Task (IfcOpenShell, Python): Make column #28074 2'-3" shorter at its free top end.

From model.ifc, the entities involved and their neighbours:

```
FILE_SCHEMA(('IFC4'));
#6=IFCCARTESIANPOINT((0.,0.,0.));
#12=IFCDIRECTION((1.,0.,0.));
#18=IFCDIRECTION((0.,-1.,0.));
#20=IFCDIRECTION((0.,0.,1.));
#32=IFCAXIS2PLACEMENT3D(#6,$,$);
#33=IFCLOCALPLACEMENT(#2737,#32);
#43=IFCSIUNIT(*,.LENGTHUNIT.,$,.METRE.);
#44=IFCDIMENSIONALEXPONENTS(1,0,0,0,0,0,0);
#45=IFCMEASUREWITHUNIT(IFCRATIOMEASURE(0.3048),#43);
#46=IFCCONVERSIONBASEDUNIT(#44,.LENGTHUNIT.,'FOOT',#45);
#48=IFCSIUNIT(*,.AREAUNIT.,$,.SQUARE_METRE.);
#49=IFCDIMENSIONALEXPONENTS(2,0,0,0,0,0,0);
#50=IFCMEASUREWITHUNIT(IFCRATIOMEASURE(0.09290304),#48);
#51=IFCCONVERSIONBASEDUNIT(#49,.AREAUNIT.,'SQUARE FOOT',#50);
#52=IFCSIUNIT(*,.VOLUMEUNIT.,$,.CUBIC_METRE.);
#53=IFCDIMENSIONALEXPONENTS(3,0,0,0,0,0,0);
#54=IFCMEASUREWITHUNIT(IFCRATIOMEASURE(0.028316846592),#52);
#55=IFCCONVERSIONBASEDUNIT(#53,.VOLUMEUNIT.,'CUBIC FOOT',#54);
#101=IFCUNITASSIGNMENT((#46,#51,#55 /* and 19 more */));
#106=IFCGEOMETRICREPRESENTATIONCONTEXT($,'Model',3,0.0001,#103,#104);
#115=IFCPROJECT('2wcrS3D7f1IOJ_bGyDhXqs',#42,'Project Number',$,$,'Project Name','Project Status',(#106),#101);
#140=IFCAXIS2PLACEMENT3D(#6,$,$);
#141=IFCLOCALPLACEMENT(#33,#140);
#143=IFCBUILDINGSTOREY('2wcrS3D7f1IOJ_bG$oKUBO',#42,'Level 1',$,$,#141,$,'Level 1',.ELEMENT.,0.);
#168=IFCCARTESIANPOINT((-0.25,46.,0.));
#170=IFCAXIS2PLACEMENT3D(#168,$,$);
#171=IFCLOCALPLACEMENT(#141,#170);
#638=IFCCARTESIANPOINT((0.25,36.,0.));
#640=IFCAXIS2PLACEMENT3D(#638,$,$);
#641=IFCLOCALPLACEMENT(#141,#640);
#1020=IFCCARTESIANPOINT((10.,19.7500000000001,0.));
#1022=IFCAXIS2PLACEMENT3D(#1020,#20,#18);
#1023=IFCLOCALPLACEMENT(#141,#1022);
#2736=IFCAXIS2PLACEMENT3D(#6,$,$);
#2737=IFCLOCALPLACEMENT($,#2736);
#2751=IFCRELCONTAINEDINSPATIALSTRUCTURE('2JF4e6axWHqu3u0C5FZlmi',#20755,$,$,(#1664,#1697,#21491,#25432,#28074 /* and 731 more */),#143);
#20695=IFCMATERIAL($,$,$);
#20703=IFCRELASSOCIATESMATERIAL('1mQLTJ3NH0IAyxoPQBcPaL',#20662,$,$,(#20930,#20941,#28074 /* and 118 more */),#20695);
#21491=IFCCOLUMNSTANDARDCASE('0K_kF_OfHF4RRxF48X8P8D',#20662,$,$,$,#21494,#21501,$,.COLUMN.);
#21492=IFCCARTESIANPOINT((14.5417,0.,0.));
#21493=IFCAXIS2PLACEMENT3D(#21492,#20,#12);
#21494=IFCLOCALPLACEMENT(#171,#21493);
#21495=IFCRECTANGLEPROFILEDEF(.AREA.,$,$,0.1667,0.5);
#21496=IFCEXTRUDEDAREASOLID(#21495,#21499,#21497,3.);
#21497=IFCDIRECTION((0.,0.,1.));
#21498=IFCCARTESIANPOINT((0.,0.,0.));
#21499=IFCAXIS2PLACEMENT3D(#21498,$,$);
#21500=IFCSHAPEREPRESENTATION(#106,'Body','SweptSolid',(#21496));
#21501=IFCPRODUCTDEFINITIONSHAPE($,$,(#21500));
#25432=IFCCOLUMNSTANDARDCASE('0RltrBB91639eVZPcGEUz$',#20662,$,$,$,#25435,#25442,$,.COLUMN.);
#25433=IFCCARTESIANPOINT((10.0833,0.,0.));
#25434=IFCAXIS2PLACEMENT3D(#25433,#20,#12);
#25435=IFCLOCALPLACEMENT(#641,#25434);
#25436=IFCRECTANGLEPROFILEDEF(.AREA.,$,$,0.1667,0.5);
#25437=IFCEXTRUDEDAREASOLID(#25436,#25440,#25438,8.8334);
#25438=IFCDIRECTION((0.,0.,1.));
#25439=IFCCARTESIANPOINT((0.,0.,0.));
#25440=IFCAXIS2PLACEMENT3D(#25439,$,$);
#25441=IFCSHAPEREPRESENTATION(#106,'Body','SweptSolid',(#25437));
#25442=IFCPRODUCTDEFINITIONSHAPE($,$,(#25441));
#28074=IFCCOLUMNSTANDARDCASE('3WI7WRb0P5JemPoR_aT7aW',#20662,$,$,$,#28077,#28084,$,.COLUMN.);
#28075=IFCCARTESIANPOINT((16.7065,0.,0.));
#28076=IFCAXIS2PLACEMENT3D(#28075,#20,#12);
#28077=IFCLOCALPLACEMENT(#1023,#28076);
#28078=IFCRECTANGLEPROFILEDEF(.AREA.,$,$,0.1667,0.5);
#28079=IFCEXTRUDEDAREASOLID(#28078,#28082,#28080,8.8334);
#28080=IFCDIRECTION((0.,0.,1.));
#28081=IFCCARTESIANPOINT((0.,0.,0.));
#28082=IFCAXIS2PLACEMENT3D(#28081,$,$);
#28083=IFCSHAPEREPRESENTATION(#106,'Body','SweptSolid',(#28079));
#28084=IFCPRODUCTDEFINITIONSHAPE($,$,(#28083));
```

```python
import ifcopenshell
import ifcopenshell.util.unit

model = ifcopenshell.open("model.ifc")
unit_scale = ifcopenshell.util.unit.calculate_unit_scale(model)

member = model.by_guid("3WI7WRb0P5JemPoR_aT7aW")
change = -27 * 0.0254 / unit_scale

# The extrusion runs towards the end named, so only its depth changes.
body = next(r for r in member.Representation.Representations if r.RepresentationIdentifier == "Body")
solid = body.Items[0]
old_length = solid.Depth
solid.Depth += change

print(f"length {old_length:g} -> {solid.Depth:g}")

model.write("model-out.ifc")
```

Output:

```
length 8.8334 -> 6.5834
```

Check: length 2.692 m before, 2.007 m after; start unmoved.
